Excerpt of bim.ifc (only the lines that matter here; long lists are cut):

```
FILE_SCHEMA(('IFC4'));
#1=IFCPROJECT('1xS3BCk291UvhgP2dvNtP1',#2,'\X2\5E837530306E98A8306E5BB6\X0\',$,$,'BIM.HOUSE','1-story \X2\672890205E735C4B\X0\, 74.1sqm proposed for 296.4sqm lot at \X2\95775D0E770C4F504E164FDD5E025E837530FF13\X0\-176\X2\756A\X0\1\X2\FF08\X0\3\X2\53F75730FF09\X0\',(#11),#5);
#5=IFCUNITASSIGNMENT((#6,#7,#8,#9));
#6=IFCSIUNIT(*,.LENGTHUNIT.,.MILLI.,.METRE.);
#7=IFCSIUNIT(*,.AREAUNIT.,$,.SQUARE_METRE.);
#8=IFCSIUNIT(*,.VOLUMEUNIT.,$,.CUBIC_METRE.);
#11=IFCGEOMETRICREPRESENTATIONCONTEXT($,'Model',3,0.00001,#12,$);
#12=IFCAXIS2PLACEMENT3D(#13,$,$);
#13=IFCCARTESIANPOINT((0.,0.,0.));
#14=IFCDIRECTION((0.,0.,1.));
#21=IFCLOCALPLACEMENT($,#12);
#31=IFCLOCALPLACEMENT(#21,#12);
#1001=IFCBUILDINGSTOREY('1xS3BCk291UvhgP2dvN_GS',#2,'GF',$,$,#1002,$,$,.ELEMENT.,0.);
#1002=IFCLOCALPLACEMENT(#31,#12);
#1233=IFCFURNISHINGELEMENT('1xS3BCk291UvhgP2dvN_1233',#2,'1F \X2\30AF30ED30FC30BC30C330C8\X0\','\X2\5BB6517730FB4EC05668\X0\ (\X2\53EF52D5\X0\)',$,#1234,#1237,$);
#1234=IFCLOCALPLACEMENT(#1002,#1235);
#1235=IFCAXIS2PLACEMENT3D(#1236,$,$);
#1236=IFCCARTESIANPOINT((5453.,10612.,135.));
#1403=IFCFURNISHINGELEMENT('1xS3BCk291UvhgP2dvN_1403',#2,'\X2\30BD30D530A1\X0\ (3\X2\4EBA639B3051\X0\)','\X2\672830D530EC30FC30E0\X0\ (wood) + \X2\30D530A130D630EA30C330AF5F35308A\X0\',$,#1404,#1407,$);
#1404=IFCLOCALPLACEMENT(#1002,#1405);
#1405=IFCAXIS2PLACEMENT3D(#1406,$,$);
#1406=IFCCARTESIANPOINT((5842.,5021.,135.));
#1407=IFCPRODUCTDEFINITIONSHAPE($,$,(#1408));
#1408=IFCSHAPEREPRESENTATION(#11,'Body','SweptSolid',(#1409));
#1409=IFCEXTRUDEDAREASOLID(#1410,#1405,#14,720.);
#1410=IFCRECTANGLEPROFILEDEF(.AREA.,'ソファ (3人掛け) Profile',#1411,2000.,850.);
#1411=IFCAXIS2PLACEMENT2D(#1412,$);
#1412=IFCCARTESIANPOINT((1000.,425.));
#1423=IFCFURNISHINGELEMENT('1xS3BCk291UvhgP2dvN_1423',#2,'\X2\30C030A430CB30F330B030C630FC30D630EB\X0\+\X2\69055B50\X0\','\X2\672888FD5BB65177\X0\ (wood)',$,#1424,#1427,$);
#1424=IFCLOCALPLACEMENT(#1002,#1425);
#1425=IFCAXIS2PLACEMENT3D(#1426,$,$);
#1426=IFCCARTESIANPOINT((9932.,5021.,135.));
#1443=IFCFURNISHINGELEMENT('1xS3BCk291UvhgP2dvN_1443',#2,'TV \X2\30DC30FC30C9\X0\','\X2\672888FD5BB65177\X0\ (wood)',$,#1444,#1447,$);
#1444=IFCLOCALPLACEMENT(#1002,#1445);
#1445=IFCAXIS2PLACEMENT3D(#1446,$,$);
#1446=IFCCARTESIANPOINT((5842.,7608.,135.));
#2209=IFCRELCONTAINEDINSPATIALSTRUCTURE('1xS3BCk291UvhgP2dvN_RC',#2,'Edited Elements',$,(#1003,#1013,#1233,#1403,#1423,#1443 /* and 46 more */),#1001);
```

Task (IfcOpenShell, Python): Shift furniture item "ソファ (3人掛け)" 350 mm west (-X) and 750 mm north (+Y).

```python
import ifcopenshell
import ifcopenshell.api.geometry
import ifcopenshell.util.placement
import ifcopenshell.util.unit

model = ifcopenshell.open("bim.ifc")
unit_scale = ifcopenshell.util.unit.calculate_unit_scale(model)

item = model.by_guid("1xS3BCk291UvhgP2dvN_1403")
matrix = ifcopenshell.util.placement.get_local_placement(item.ObjectPlacement)
matrix[0, 3] -= 0.35 / unit_scale
matrix[1, 3] += 0.75 / unit_scale
ifcopenshell.api.geometry.edit_object_placement(model, product=item, matrix=matrix, is_si=False)

print(ifcopenshell.util.placement.get_local_placement(item.ObjectPlacement).round(3) + 0.0)

model.write("bim_v2.ifc")
```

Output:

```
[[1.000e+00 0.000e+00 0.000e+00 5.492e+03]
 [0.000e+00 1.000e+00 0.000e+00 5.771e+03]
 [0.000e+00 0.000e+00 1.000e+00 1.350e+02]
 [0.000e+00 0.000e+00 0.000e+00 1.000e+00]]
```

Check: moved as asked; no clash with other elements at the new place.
